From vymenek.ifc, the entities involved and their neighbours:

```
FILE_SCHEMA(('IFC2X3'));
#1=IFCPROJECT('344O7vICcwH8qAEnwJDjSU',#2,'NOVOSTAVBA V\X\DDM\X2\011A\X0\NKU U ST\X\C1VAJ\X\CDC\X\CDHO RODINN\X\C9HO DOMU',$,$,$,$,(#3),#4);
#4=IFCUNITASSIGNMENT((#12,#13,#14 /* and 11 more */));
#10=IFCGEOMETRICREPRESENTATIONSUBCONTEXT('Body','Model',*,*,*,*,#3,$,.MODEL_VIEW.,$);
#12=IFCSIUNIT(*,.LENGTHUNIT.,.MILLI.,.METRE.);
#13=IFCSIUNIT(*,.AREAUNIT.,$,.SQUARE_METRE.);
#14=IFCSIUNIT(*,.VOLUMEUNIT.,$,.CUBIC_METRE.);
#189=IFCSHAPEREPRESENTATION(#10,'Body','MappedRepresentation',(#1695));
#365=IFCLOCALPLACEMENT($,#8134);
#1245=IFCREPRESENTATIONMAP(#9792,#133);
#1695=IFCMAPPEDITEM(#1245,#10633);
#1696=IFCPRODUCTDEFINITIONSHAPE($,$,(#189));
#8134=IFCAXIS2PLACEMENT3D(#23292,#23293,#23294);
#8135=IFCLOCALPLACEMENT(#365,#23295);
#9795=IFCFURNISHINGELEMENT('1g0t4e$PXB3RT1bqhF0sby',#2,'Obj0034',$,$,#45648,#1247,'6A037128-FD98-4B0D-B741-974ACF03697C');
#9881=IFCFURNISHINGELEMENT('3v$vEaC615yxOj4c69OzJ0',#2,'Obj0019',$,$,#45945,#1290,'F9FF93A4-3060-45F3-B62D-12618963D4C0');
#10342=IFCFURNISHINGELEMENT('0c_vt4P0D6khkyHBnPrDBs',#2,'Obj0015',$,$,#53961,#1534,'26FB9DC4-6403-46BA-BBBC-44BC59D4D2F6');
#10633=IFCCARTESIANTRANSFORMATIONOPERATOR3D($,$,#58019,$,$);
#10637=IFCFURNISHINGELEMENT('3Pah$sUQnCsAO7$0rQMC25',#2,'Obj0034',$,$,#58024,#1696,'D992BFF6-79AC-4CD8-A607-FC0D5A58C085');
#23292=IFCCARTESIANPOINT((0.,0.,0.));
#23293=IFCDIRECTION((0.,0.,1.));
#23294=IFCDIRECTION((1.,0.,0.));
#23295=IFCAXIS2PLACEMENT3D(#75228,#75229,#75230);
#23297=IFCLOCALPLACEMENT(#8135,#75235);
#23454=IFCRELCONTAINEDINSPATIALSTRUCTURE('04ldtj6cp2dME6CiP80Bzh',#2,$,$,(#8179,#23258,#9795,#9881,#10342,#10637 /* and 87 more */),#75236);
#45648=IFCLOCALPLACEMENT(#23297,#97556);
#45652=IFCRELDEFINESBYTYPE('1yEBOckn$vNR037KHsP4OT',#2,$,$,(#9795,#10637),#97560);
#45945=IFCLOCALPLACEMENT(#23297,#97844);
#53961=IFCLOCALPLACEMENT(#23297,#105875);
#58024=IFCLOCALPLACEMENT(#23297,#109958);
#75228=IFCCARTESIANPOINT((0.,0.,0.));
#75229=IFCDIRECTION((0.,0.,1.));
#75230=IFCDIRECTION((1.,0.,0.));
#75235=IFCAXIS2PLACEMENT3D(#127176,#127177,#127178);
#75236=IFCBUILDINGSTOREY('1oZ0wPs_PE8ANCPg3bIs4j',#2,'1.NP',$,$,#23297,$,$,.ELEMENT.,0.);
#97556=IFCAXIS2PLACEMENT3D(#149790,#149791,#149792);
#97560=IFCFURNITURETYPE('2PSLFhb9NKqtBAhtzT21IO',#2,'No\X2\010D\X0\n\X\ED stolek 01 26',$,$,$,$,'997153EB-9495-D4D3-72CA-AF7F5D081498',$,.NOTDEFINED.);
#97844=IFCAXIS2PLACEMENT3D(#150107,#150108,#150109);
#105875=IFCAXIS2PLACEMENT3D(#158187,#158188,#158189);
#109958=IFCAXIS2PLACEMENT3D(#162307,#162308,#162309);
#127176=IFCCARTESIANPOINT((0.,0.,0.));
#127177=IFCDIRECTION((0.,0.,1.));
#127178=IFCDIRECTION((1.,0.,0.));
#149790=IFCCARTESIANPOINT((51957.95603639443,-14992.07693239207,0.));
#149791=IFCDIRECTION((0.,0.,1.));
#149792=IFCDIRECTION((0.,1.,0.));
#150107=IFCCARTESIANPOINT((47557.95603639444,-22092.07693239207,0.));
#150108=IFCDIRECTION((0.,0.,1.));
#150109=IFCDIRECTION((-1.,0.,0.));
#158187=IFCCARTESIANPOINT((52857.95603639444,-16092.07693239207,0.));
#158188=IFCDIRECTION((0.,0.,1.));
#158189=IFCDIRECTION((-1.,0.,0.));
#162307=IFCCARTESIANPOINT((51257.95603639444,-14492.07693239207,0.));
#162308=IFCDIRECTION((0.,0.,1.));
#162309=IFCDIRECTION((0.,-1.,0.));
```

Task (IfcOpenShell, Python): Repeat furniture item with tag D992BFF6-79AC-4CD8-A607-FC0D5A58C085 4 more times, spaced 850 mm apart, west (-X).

```python
import numpy as np
import ifcopenshell
import ifcopenshell.api.geometry
import ifcopenshell.api.root
import ifcopenshell.util.element
import ifcopenshell.util.placement

model = ifcopenshell.open("vymenek.ifc")


def reuse_history(source, copy):
    """copy_class also copies each property set's owner history, people and application; keep the originals."""
    for rel in copy.IsDefinedBy:
        if rel.is_a("IfcRelDefinesByProperties") and (history := rel.RelatingPropertyDefinition.OwnerHistory):
            rel.RelatingPropertyDefinition.OwnerHistory = source.OwnerHistory
            ifcopenshell.util.element.remove_deep2(model, history)


source = model.by_guid("3Pah$sUQnCsAO7$0rQMC25")
base = ifcopenshell.util.placement.get_local_placement(source.ObjectPlacement)
step = np.array([-1.0, 0.0, 0.0]) * 850.0

for i in range(1, 5):
    copy = ifcopenshell.api.root.copy_class(model, product=source)
    copy.Representation = ifcopenshell.util.element.copy_deep(
        model, source.Representation, exclude=["IfcGeometricRepresentationContext", "IfcRepresentationMap"]
    )
    copy.Tag = None
    reuse_history(source, copy)
    matrix = base.copy()
    matrix[:3, 3] += i * step
    print("added at", matrix[:3, 3].round(3) + 0.0)
    ifcopenshell.api.geometry.edit_object_placement(model, product=copy, matrix=matrix, is_si=False)

model.write("vymenek_updated.ifc")
```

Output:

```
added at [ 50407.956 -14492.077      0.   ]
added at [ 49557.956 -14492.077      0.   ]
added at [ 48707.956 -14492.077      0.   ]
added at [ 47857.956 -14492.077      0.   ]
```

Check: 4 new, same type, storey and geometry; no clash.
